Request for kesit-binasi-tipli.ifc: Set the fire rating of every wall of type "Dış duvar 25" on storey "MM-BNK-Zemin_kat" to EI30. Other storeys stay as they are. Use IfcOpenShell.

First a look at what the model holds.

```python
import ifcopenshell
import ifcopenshell.util.element

model = ifcopenshell.open("kesit-binasi-tipli.ifc")
print(model.schema)
storey = next(s for s in model.by_type("IfcBuildingStorey") if s.Name == "MM-BNK-Zemin_kat")
walls = [e for e in ifcopenshell.util.element.get_decomposition(storey) if e.is_a("IfcWall")]
seen = {}
for e in walls:
    element_type = ifcopenshell.util.element.get_type(e)
    key = (element_type.Name if element_type != e and element_type else None, ifcopenshell.util.element.get_pset(e, "Pset_WallCommon", "FireRating"))
    seen[key] = seen.get(key, 0) + 1
for (name, value), count in sorted(seen.items(), key=str):
    print(count, "x", name, "|", value)
```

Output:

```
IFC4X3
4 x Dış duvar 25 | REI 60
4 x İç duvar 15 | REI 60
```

```python
import ifcopenshell
import ifcopenshell.api.pset
import ifcopenshell.util.element

model = ifcopenshell.open("kesit-binasi-tipli.ifc")

storey = next(s for s in model.by_type("IfcBuildingStorey") if s.Name == "MM-BNK-Zemin_kat")
walls = [e for e in ifcopenshell.util.element.get_decomposition(storey) if e.is_a("IfcWall")]

count = 0
for e in walls:
    element_type = ifcopenshell.util.element.get_type(e)
    if element_type in (None, e) or element_type.Name != "Dış duvar 25":
        continue
    # add_pset returns the element's existing set when there is one.
    pset = ifcopenshell.api.pset.add_pset(model, product=e, name="Pset_WallCommon")
    ifcopenshell.api.pset.edit_pset(model, pset=pset, properties={"FireRating": "EI30"})
    count += 1

print(count, "walls updated")

model.write("kesit-binasi-tipli_edited.ifc")
```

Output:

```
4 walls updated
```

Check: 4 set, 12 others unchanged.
